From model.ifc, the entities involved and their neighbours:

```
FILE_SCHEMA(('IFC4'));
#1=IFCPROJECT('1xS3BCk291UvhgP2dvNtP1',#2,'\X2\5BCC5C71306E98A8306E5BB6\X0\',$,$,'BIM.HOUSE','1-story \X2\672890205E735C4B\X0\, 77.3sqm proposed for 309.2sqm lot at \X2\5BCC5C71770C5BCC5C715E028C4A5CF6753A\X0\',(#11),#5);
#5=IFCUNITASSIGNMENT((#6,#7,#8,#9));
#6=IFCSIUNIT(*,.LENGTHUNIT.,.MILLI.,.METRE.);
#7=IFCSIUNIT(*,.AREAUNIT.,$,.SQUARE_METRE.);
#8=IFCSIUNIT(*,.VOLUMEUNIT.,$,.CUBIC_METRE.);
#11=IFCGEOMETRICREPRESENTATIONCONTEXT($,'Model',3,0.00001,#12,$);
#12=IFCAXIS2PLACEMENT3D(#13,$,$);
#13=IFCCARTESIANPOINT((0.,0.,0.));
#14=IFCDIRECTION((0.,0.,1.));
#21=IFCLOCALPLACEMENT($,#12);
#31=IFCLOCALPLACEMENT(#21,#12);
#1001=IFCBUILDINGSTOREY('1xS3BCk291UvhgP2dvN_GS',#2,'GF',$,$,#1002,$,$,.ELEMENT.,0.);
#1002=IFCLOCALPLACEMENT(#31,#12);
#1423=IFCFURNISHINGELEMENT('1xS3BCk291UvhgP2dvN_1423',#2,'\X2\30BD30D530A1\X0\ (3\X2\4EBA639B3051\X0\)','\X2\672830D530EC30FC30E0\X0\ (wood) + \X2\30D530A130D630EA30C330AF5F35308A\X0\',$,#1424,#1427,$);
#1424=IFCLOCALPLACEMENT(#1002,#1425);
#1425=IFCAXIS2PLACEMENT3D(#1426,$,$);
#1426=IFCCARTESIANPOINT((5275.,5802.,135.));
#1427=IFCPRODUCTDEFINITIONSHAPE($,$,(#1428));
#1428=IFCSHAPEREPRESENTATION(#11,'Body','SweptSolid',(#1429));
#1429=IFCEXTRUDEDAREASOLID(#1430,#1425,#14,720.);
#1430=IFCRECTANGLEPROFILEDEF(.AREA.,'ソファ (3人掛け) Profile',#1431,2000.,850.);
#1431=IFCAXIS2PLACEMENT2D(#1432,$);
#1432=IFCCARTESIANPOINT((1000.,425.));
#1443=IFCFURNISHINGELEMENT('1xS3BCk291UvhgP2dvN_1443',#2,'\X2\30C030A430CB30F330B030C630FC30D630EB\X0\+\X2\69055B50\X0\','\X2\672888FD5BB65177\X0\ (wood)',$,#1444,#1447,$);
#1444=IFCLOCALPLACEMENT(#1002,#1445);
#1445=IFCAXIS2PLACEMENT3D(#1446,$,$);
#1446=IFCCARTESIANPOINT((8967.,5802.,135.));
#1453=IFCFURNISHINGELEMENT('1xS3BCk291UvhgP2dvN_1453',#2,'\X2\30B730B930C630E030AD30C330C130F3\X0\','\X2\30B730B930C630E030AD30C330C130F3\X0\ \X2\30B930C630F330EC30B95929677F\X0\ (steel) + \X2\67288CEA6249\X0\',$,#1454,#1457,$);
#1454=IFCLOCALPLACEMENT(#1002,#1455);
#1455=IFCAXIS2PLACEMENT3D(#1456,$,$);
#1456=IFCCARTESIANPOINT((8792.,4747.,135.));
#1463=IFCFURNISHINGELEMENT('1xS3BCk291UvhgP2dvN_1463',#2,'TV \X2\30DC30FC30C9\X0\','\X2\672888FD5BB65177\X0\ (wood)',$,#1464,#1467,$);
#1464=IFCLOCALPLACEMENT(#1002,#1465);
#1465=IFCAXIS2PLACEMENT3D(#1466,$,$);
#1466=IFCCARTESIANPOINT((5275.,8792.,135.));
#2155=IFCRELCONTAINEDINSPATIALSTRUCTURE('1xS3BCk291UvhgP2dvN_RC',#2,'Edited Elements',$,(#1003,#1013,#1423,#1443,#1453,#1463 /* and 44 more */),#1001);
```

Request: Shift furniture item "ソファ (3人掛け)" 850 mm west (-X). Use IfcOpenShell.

```python
import ifcopenshell
import ifcopenshell.api.geometry
import ifcopenshell.util.placement

model = ifcopenshell.open("model.ifc")

item = model.by_id(1423)
matrix = ifcopenshell.util.placement.get_local_placement(item.ObjectPlacement)
matrix[0, 3] -= 850.0
ifcopenshell.api.geometry.edit_object_placement(model, product=item, matrix=matrix, is_si=False)

print(ifcopenshell.util.placement.get_local_placement(item.ObjectPlacement).round(3) + 0.0)

model.write("model_edited.ifc")
```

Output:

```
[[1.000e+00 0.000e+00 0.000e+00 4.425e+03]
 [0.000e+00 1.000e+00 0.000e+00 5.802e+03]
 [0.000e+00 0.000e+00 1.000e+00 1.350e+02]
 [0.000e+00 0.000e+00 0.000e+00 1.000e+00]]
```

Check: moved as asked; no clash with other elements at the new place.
